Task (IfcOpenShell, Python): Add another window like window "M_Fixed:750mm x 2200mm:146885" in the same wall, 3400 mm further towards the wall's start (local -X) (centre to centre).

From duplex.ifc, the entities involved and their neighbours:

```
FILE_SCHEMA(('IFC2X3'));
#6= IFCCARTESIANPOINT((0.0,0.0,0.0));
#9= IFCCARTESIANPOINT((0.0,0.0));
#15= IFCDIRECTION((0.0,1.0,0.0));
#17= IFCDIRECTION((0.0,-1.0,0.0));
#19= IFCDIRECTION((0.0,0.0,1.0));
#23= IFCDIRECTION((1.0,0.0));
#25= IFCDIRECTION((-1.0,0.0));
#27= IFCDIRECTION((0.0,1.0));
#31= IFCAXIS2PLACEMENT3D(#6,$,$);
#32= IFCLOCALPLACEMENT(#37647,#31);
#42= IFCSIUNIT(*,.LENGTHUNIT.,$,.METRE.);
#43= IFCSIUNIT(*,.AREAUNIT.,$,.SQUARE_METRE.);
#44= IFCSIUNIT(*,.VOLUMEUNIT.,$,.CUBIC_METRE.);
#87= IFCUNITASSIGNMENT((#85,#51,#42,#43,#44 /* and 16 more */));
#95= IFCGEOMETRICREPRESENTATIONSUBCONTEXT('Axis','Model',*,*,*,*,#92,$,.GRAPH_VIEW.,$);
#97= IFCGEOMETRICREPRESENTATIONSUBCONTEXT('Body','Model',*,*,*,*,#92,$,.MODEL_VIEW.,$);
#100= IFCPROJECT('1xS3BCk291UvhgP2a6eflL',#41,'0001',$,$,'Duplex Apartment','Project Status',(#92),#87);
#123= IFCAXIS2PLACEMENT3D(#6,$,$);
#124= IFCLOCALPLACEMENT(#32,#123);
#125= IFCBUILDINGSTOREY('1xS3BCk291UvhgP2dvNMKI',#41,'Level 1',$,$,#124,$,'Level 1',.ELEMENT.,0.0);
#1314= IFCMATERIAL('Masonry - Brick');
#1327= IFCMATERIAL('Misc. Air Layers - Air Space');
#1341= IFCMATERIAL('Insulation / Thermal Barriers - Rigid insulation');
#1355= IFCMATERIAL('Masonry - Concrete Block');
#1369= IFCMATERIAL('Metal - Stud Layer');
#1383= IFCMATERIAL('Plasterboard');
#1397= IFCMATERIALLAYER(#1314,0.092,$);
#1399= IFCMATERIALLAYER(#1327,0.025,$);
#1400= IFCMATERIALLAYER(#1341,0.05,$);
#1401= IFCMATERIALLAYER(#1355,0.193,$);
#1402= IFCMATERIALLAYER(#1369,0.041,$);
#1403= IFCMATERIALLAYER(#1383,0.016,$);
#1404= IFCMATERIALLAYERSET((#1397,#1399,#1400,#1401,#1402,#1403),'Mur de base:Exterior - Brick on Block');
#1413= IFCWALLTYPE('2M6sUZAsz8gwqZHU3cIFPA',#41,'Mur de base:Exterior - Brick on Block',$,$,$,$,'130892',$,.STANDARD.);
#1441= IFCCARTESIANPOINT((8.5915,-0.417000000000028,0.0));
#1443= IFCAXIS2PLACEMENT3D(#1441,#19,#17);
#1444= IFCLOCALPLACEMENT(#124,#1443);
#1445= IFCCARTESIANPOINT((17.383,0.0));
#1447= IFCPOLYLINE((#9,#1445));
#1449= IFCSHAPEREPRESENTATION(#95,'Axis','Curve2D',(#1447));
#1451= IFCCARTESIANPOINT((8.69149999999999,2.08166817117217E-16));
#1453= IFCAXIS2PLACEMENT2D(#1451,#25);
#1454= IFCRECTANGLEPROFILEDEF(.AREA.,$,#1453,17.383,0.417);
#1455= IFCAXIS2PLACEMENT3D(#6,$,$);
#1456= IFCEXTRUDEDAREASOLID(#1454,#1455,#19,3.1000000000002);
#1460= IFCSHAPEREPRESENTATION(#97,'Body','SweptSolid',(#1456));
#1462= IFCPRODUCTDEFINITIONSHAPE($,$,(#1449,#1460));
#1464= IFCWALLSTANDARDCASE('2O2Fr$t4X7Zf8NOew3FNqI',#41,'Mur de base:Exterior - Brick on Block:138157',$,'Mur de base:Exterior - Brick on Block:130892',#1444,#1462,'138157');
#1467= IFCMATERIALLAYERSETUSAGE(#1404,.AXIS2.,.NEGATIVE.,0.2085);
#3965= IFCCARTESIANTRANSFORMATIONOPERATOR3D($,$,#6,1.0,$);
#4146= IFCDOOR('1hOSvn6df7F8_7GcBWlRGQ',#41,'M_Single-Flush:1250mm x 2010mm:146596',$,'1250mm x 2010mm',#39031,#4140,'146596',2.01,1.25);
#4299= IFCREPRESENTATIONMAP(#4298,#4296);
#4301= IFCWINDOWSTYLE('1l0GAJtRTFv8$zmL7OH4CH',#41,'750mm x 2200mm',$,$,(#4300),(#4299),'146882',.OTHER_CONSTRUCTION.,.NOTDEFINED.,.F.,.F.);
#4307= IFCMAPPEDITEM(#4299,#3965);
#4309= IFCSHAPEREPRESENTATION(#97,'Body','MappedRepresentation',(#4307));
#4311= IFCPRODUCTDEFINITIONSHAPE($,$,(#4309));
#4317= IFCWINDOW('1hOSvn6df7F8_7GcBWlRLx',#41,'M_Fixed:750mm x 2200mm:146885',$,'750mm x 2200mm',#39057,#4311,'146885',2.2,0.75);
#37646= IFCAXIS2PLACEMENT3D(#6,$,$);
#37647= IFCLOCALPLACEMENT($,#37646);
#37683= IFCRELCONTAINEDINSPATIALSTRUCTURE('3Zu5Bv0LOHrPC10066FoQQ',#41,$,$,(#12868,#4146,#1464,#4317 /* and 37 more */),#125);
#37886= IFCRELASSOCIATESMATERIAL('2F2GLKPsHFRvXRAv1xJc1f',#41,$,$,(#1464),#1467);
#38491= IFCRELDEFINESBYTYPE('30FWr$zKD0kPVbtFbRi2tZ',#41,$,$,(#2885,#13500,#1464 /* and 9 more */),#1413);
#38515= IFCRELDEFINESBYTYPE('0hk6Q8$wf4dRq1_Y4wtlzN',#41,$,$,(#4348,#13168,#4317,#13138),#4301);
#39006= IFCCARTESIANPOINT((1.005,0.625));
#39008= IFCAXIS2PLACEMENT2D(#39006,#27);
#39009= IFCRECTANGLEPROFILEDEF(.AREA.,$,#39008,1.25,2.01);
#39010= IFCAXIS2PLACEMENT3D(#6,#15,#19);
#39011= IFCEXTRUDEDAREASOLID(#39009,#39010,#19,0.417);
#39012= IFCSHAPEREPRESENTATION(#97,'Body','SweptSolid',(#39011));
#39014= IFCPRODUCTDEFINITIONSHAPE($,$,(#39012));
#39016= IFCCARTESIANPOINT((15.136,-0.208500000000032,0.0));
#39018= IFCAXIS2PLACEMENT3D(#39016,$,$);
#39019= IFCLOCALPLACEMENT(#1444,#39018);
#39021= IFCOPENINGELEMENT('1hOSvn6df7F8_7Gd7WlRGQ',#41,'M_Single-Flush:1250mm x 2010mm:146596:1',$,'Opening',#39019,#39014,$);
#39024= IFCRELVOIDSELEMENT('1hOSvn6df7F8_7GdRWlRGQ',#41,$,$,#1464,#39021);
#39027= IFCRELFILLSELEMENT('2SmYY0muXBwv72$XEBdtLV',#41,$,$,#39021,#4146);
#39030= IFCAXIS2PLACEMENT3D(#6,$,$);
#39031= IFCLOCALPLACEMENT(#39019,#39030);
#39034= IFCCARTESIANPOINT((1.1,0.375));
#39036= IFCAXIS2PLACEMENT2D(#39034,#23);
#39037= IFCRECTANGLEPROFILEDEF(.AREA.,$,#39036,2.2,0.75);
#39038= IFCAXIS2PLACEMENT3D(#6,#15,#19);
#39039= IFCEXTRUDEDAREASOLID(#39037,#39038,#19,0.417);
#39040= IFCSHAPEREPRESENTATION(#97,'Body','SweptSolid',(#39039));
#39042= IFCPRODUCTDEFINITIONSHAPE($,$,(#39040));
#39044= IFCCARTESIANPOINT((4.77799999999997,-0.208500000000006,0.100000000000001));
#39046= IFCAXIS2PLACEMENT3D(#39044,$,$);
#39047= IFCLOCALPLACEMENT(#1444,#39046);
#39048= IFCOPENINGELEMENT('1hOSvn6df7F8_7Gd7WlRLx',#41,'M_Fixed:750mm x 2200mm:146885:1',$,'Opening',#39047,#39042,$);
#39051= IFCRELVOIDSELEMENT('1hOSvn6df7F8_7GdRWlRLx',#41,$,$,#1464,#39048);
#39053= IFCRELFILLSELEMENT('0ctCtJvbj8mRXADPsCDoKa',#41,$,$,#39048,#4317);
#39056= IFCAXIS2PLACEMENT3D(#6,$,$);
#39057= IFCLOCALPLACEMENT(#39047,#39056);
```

```python
import ifcopenshell
import ifcopenshell.api.feature
import ifcopenshell.api.geometry
import ifcopenshell.api.root
import ifcopenshell.geom
import ifcopenshell.util.element
import ifcopenshell.util.placement
import ifcopenshell.util.shape
import ifcopenshell.util.unit

model = ifcopenshell.open("duplex.ifc")
unit_scale = ifcopenshell.util.unit.calculate_unit_scale(model)
settings = ifcopenshell.geom.settings()


def volume(element):
    """Net volume in cubic metres, openings subtracted."""
    shape = ifcopenshell.geom.create_shape(settings, element)
    return ifcopenshell.util.shape.get_volume(shape.geometry)


def reuse_history(source, copy):
    """copy_class also copies each property set's owner history, people and application; keep the originals."""
    for rel in copy.IsDefinedBy:
        if rel.is_a("IfcRelDefinesByProperties") and (history := rel.RelatingPropertyDefinition.OwnerHistory):
            rel.RelatingPropertyDefinition.OwnerHistory = source.OwnerHistory
            ifcopenshell.util.element.remove_deep2(model, history)


window = model.by_guid("1hOSvn6df7F8_7GcBWlRLx")
opening = window.FillsVoids[0].RelatingOpeningElement
wall = opening.VoidsElements[0].RelatingBuildingElement
before = volume(wall)
shift = ifcopenshell.util.placement.get_local_placement(wall.ObjectPlacement)[:3, 0] * -3.4 / unit_scale

# copy_class copies the void relationship, type, container and properties, but no geometry.
new_opening = ifcopenshell.api.root.copy_class(model, product=opening)
new_opening.Representation = ifcopenshell.util.element.copy_deep(
    model, opening.Representation, exclude=["IfcGeometricRepresentationContext", "IfcRepresentationMap"]
)
new_opening.Name = "M_Fixed:750mm x 2200mm"
new_window = ifcopenshell.api.root.copy_class(model, product=window)
new_window.Representation = ifcopenshell.util.element.copy_deep(
    model, window.Representation, exclude=["IfcGeometricRepresentationContext", "IfcRepresentationMap"]
)
new_window.Name = "M_Fixed:750mm x 2200mm"
new_window.Tag = None
reuse_history(window, new_window)
fills = ifcopenshell.api.feature.add_filling(model, opening=new_opening, element=new_window)
fills.OwnerHistory = new_window.OwnerHistory  # required in IFC2X3

for old, new in ((opening, new_opening), (window, new_window)):
    matrix = ifcopenshell.util.placement.get_local_placement(old.ObjectPlacement)
    matrix[:3, 3] += shift
    ifcopenshell.api.geometry.edit_object_placement(model, product=new, matrix=matrix, is_si=False)

after = volume(wall)

print(f"wall volume {before:.3f} -> {after:.3f} m3")

model.write("duplex_edited.ifc")
```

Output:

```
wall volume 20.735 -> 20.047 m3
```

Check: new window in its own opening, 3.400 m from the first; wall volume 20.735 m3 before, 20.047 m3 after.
